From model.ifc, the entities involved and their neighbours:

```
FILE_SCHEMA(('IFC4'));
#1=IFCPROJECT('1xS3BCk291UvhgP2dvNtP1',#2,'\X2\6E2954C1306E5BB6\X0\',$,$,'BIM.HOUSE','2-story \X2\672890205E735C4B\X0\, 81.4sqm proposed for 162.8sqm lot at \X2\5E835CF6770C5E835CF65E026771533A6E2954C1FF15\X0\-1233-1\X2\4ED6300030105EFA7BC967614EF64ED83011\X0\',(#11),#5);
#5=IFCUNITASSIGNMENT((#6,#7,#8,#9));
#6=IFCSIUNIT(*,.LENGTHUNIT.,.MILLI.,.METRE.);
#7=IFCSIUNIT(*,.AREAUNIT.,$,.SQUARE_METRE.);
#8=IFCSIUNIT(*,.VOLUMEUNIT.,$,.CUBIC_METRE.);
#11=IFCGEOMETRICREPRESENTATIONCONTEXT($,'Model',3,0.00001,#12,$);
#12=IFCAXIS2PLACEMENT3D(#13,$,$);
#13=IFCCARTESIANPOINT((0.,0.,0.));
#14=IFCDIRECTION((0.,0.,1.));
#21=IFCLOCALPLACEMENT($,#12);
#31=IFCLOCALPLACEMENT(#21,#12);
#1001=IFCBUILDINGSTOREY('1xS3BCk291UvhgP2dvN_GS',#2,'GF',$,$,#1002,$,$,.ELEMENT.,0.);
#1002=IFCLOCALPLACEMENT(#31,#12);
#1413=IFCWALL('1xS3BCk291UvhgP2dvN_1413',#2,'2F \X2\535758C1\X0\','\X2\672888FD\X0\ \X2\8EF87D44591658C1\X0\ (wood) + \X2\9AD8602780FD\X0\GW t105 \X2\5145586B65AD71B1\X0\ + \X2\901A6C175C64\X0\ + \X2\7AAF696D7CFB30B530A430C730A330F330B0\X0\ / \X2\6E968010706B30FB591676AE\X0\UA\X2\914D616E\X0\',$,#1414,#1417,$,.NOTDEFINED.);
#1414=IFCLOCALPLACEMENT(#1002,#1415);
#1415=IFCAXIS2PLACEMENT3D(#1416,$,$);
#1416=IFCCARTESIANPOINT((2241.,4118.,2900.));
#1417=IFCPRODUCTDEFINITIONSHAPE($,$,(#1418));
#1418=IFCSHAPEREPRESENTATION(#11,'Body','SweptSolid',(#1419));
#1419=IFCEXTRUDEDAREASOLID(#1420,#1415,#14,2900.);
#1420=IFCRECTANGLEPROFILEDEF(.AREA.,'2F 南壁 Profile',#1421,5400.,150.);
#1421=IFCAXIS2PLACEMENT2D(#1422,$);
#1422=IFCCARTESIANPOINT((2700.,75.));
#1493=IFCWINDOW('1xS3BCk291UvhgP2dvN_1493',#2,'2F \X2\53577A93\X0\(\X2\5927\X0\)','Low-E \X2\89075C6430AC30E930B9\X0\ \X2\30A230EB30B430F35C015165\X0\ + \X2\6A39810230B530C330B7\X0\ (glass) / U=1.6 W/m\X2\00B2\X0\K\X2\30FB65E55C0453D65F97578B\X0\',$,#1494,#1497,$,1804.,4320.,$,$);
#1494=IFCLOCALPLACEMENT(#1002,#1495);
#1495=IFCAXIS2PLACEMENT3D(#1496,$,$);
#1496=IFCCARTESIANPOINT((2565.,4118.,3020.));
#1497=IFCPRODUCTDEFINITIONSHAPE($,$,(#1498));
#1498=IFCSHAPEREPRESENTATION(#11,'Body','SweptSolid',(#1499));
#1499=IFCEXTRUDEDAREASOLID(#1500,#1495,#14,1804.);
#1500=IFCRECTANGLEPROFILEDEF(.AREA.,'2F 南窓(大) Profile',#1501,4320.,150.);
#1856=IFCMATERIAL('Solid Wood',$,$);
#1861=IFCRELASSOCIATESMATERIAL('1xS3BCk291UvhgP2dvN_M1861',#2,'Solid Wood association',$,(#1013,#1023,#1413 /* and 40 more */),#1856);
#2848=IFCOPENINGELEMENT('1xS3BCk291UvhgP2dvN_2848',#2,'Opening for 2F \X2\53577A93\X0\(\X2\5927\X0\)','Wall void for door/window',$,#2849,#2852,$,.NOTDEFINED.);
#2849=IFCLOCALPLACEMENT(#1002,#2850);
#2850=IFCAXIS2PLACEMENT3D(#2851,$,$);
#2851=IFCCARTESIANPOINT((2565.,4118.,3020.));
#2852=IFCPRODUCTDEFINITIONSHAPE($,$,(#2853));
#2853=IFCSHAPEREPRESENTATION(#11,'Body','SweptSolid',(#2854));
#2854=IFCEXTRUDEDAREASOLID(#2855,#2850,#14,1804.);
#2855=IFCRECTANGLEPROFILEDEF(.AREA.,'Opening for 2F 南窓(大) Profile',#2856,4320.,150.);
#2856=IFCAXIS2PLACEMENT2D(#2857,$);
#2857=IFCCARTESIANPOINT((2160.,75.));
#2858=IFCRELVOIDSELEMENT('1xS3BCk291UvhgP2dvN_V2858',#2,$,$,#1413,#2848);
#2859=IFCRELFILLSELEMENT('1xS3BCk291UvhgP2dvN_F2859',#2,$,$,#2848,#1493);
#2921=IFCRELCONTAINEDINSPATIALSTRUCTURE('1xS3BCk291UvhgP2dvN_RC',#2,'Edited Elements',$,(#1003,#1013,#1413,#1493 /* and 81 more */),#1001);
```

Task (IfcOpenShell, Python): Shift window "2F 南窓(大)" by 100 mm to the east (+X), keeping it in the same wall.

```python
import ifcopenshell
import ifcopenshell.api.geometry
import ifcopenshell.util.placement

model = ifcopenshell.open("model.ifc")

window = model.by_guid("1xS3BCk291UvhgP2dvN_1493")
opening = window.FillsVoids[0].RelatingOpeningElement
wall = opening.VoidsElements[0].RelatingBuildingElement

wall_matrix = ifcopenshell.util.placement.get_local_placement(wall.ObjectPlacement)
shift = wall_matrix[:3, 0] * 100.0
before = ifcopenshell.util.placement.get_local_placement(window.ObjectPlacement)[:3, 3].copy()

# The window is not placed relative to its opening, so move both.
for product in (opening, window):
    matrix = ifcopenshell.util.placement.get_local_placement(product.ObjectPlacement)
    matrix[:3, 3] += shift
    ifcopenshell.api.geometry.edit_object_placement(model, product=product, matrix=matrix, is_si=False)

after = ifcopenshell.util.placement.get_local_placement(window.ObjectPlacement)[:3, 3]
print("window moved by", (after - before).round(3) + 0.0)

model.write("model_rev.ifc")
```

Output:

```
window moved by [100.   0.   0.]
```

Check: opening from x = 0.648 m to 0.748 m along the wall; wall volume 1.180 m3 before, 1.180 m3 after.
